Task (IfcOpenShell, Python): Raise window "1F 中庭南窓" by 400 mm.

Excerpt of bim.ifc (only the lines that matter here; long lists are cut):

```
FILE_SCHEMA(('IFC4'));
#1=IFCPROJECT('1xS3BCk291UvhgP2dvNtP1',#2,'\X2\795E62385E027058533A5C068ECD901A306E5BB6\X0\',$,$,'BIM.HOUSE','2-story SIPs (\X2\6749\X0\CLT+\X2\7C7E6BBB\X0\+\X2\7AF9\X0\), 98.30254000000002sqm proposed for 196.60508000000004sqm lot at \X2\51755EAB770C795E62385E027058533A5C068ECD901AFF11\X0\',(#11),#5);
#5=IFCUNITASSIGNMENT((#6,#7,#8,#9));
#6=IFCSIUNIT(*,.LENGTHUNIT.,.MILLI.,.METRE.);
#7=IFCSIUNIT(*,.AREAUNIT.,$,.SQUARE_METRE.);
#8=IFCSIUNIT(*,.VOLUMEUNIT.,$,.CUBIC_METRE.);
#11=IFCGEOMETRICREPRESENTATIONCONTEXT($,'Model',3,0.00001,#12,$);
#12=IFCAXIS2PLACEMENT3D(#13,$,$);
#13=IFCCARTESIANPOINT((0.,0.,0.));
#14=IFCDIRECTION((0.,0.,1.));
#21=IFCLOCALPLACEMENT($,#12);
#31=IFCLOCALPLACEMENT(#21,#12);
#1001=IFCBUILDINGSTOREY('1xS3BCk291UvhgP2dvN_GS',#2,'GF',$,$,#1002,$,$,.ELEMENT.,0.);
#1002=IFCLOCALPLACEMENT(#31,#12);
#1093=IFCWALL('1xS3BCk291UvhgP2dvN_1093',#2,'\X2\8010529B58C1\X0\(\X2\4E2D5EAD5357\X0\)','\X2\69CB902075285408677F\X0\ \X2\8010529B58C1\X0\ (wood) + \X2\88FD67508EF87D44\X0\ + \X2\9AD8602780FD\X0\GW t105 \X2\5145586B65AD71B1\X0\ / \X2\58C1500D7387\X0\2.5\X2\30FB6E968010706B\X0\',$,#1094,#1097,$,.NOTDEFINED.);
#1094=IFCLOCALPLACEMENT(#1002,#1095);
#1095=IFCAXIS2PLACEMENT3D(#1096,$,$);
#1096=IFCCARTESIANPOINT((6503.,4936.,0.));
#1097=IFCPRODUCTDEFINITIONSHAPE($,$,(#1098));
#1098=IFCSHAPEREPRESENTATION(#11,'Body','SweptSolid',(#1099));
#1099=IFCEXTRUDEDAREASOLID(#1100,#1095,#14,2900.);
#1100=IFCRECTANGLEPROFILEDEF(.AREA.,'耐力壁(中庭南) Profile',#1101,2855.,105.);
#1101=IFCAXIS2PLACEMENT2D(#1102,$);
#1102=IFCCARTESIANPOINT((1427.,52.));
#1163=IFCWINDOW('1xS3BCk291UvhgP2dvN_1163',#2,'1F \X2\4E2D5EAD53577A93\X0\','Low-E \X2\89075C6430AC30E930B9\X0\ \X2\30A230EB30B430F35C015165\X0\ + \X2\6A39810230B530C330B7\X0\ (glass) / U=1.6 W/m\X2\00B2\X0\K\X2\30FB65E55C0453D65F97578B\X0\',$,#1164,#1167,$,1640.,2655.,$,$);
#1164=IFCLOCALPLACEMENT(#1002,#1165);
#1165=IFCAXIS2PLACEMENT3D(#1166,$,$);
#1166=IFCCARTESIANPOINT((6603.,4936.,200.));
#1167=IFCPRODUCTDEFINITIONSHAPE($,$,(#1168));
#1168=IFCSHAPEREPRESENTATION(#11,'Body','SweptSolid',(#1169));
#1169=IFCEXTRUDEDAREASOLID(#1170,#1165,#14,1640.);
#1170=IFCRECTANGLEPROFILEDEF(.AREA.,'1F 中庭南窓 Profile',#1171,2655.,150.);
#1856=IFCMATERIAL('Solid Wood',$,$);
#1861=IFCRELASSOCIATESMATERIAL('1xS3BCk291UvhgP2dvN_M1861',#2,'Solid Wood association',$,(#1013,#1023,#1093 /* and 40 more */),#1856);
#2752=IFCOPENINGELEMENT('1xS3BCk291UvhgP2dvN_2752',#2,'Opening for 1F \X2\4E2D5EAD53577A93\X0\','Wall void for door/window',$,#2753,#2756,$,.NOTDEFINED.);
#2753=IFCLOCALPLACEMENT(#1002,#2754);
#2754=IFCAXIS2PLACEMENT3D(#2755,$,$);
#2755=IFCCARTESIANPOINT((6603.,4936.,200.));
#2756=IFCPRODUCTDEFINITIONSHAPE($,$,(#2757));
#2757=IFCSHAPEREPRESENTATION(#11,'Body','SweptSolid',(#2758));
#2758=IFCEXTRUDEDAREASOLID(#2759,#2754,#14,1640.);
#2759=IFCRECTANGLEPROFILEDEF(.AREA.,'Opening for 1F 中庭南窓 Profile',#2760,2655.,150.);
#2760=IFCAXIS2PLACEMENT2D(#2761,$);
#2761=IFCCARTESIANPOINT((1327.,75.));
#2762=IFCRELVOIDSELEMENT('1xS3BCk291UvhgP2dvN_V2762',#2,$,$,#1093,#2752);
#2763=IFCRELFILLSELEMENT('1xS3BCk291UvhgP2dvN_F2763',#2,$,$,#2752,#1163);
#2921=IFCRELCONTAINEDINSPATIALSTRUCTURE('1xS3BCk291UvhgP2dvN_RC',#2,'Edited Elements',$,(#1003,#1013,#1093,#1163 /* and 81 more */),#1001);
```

```python
import numpy as np
import ifcopenshell
import ifcopenshell.api.geometry
import ifcopenshell.util.placement
import ifcopenshell.util.unit

model = ifcopenshell.open("bim.ifc")
unit_scale = ifcopenshell.util.unit.calculate_unit_scale(model)

window = model.by_id(1163)
opening = window.FillsVoids[0].RelatingOpeningElement
dz = 0.4 / unit_scale

shift = np.array([0.0, 0.0, dz])
# The window is not placed relative to its opening, so move both.
for product in (opening, window):
    matrix = ifcopenshell.util.placement.get_local_placement(product.ObjectPlacement)
    matrix[:3, 3] += shift
    ifcopenshell.api.geometry.edit_object_placement(model, product=product, matrix=matrix, is_si=False)

print(f"moved by {dz * unit_scale:+.3f} m")

model.write("bim_updated.ifc")
```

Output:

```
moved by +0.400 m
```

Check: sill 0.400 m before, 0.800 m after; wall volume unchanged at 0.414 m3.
